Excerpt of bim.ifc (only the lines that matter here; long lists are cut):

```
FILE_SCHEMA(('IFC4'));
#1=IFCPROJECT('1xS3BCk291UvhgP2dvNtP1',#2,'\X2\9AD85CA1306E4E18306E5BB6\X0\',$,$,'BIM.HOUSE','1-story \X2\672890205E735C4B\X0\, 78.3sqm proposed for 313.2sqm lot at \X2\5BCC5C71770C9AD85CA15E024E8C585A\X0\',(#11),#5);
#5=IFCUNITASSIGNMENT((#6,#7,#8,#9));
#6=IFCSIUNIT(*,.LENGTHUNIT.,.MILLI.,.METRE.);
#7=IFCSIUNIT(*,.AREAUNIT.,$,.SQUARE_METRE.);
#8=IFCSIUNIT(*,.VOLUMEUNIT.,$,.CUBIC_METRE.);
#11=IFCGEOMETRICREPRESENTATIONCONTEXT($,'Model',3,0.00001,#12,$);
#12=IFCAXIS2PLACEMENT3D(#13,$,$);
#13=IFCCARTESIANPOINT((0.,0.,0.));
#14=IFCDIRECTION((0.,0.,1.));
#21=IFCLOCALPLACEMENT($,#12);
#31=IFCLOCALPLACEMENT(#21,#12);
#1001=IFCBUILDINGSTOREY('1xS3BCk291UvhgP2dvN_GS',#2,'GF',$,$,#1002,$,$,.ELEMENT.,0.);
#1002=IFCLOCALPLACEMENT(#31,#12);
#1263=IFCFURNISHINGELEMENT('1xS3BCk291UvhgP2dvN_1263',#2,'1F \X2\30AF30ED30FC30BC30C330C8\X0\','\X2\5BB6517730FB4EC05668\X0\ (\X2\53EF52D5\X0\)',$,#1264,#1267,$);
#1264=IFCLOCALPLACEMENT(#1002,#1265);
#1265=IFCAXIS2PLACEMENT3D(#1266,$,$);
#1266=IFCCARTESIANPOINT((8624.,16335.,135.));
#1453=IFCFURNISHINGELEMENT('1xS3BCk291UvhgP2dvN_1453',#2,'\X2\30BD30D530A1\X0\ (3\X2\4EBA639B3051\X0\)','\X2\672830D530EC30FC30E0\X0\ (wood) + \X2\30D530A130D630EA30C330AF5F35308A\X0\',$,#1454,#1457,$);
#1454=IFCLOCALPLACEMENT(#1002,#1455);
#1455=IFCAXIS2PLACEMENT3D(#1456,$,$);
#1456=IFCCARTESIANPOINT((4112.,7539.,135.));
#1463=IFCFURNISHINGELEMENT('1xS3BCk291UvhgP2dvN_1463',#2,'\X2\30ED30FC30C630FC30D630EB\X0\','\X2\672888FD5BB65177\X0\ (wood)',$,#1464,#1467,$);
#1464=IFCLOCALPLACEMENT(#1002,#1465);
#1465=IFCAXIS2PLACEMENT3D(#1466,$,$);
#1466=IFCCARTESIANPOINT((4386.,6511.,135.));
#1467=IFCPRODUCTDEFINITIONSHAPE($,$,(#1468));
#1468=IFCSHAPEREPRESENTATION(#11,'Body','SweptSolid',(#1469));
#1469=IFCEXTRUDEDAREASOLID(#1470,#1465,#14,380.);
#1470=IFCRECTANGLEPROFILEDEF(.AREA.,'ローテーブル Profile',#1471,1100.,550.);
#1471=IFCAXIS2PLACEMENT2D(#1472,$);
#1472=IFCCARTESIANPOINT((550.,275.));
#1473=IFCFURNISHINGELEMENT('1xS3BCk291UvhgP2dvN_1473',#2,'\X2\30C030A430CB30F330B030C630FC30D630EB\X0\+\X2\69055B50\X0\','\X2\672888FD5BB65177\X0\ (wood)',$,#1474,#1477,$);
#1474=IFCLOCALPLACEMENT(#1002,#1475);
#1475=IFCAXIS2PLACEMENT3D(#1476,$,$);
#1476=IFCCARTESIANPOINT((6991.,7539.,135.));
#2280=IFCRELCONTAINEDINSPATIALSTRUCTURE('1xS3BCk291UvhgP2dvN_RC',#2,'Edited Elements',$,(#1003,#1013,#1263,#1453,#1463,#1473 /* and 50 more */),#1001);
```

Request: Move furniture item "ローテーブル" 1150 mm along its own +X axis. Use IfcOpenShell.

```python
import ifcopenshell
import ifcopenshell.api.geometry
import ifcopenshell.util.placement
import ifcopenshell.util.unit

model = ifcopenshell.open("bim.ifc")
unit_scale = ifcopenshell.util.unit.calculate_unit_scale(model)

item = model.by_id(1463)
matrix = ifcopenshell.util.placement.get_local_placement(item.ObjectPlacement)
matrix[:3, 3] += matrix[:3, 0] * 1.15 / unit_scale
ifcopenshell.api.geometry.edit_object_placement(model, product=item, matrix=matrix, is_si=False)

print(ifcopenshell.util.placement.get_local_placement(item.ObjectPlacement).round(3) + 0.0)

model.write("bim-out.ifc")
```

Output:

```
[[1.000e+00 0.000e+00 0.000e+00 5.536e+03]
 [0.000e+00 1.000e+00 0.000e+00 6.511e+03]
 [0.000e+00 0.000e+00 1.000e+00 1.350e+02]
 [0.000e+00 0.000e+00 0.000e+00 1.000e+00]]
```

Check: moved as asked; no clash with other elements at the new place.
